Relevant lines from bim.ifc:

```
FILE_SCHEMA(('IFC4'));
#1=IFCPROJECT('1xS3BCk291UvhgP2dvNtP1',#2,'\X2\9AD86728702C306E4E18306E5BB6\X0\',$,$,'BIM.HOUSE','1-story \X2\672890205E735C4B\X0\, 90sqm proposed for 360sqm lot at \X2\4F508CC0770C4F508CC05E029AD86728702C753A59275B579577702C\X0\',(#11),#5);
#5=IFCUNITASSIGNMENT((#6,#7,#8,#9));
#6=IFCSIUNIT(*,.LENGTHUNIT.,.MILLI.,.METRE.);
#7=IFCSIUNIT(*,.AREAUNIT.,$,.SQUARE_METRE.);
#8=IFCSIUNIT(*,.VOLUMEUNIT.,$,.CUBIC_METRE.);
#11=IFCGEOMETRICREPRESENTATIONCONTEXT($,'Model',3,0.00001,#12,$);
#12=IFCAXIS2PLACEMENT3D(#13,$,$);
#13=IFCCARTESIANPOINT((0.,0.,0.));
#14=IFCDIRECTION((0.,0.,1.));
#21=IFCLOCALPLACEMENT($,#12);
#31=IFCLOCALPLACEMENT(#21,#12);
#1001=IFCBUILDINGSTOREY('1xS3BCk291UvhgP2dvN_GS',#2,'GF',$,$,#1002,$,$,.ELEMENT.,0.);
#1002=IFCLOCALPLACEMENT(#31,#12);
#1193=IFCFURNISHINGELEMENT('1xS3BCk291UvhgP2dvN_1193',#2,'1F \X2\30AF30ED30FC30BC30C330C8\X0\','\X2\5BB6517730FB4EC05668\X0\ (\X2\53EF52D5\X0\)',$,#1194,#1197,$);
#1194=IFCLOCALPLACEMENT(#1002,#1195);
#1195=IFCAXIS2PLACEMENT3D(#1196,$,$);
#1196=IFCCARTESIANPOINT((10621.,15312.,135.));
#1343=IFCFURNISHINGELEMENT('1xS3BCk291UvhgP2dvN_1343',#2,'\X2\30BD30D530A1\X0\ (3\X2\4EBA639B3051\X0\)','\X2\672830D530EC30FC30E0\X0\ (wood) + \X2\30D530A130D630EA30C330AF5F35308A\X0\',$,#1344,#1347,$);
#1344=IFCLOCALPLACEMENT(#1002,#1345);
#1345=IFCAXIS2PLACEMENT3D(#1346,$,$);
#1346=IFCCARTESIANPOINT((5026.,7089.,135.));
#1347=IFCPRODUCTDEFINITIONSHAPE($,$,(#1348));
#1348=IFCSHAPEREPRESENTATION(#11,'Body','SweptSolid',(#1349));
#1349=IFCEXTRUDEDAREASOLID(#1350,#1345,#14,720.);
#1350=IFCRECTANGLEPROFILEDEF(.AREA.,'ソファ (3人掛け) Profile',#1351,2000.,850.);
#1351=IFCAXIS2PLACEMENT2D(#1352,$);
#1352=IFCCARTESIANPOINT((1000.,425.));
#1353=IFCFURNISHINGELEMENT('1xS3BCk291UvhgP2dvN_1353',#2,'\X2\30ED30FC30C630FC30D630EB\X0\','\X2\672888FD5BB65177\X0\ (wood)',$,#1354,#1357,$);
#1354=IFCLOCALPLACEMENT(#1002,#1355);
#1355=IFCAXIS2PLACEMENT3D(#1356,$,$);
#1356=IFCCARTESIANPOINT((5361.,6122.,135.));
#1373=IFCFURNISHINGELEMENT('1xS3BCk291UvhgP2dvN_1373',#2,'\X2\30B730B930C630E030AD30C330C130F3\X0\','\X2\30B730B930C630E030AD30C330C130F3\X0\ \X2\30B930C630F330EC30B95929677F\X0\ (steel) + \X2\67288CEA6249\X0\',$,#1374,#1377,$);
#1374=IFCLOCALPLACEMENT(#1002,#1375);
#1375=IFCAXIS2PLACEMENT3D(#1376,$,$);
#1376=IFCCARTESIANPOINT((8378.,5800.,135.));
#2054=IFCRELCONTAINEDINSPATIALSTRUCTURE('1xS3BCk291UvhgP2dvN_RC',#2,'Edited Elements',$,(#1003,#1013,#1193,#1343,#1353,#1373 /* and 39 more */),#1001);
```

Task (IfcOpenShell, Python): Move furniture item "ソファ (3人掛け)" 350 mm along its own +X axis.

```python
import ifcopenshell
import ifcopenshell.api.geometry
import ifcopenshell.util.placement
import ifcopenshell.util.unit

model = ifcopenshell.open("bim.ifc")
unit_scale = ifcopenshell.util.unit.calculate_unit_scale(model)

item = model.by_guid("1xS3BCk291UvhgP2dvN_1343")
matrix = ifcopenshell.util.placement.get_local_placement(item.ObjectPlacement)
matrix[:3, 3] += matrix[:3, 0] * 0.35 / unit_scale
ifcopenshell.api.geometry.edit_object_placement(model, product=item, matrix=matrix, is_si=False)

print(ifcopenshell.util.placement.get_local_placement(item.ObjectPlacement).round(3) + 0.0)

model.write("bim_updated.ifc")
```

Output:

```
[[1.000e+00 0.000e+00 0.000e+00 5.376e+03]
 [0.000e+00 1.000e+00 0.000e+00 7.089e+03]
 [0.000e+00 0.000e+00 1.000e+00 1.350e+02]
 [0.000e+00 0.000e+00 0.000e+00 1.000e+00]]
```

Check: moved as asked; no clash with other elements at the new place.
